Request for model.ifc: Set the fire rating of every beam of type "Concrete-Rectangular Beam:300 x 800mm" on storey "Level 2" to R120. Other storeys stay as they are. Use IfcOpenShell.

First a look at what the model holds.

```python
import ifcopenshell
import ifcopenshell.util.element

model = ifcopenshell.open("model.ifc")
print(model.schema)
storey = next(s for s in model.by_type("IfcBuildingStorey") if s.Name == "Level 2")
beams = [e for e in ifcopenshell.util.element.get_decomposition(storey) if e.is_a("IfcBeam")]
seen = {}
for e in beams:
    element_type = ifcopenshell.util.element.get_type(e)
    key = (element_type.Name if element_type != e and element_type else None, ifcopenshell.util.element.get_pset(e, "Pset_BeamCommon", "FireRating"))
    seen[key] = seen.get(key, 0) + 1
for (name, value), count in sorted(seen.items(), key=str):
    print(count, "x", name, "|", value)
```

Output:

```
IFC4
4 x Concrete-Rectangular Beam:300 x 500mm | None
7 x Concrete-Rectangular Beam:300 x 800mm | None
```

```python
import ifcopenshell
import ifcopenshell.api.pset
import ifcopenshell.util.element

model = ifcopenshell.open("model.ifc")

storey = next(s for s in model.by_type("IfcBuildingStorey") if s.Name == "Level 2")
beams = [e for e in ifcopenshell.util.element.get_decomposition(storey) if e.is_a("IfcBeam")]

count = 0
for e in beams:
    element_type = ifcopenshell.util.element.get_type(e)
    if element_type in (None, e) or element_type.Name != "Concrete-Rectangular Beam:300 x 800mm":
        continue
    # add_pset returns the element's existing set when there is one.
    pset = ifcopenshell.api.pset.add_pset(model, product=e, name="Pset_BeamCommon")
    ifcopenshell.api.pset.edit_pset(model, pset=pset, properties={"FireRating": "R120"})
    count += 1

print(count, "beams updated")

model.write("model_v2.ifc")
```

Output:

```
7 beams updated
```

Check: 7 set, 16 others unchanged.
